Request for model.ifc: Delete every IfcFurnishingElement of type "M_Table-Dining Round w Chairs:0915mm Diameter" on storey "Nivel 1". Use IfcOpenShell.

First a look at what the model holds.

```python
import ifcopenshell
import ifcopenshell.util.element

model = ifcopenshell.open("model.ifc")
print(model.schema)
storey = next(s for s in model.by_type("IfcBuildingStorey") if s.Name == "Nivel 1")
furniture = [e for e in ifcopenshell.util.element.get_decomposition(storey) if e.is_a("IfcFurnishingElement")]
seen = {}
for e in furniture:
    element_type = ifcopenshell.util.element.get_type(e)
    name = element_type.Name if element_type not in (None, e) else None
    seen[name] = seen.get(name, 0) + 1
for name, count in sorted(seen.items(), key=str):
    print(count, "x", name)
```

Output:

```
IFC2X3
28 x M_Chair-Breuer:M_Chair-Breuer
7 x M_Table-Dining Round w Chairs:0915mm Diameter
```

```python
import ifcopenshell
import ifcopenshell.api.root
import ifcopenshell.util.element

model = ifcopenshell.open("model.ifc")

storey = next(s for s in model.by_type("IfcBuildingStorey") if s.Name == "Nivel 1")
furniture = [e for e in ifcopenshell.util.element.get_decomposition(storey) if e.is_a("IfcFurnishingElement")]
targets = [e for e in furniture if (t := ifcopenshell.util.element.get_type(e)) not in (None, e) and t.Name == "M_Table-Dining Round w Chairs:0915mm Diameter"]

for e in targets:
    ifcopenshell.api.root.remove_product(model, product=e)
print(len(targets), "removed")

model.write("model_v2.ifc")
```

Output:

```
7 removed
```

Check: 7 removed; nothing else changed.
